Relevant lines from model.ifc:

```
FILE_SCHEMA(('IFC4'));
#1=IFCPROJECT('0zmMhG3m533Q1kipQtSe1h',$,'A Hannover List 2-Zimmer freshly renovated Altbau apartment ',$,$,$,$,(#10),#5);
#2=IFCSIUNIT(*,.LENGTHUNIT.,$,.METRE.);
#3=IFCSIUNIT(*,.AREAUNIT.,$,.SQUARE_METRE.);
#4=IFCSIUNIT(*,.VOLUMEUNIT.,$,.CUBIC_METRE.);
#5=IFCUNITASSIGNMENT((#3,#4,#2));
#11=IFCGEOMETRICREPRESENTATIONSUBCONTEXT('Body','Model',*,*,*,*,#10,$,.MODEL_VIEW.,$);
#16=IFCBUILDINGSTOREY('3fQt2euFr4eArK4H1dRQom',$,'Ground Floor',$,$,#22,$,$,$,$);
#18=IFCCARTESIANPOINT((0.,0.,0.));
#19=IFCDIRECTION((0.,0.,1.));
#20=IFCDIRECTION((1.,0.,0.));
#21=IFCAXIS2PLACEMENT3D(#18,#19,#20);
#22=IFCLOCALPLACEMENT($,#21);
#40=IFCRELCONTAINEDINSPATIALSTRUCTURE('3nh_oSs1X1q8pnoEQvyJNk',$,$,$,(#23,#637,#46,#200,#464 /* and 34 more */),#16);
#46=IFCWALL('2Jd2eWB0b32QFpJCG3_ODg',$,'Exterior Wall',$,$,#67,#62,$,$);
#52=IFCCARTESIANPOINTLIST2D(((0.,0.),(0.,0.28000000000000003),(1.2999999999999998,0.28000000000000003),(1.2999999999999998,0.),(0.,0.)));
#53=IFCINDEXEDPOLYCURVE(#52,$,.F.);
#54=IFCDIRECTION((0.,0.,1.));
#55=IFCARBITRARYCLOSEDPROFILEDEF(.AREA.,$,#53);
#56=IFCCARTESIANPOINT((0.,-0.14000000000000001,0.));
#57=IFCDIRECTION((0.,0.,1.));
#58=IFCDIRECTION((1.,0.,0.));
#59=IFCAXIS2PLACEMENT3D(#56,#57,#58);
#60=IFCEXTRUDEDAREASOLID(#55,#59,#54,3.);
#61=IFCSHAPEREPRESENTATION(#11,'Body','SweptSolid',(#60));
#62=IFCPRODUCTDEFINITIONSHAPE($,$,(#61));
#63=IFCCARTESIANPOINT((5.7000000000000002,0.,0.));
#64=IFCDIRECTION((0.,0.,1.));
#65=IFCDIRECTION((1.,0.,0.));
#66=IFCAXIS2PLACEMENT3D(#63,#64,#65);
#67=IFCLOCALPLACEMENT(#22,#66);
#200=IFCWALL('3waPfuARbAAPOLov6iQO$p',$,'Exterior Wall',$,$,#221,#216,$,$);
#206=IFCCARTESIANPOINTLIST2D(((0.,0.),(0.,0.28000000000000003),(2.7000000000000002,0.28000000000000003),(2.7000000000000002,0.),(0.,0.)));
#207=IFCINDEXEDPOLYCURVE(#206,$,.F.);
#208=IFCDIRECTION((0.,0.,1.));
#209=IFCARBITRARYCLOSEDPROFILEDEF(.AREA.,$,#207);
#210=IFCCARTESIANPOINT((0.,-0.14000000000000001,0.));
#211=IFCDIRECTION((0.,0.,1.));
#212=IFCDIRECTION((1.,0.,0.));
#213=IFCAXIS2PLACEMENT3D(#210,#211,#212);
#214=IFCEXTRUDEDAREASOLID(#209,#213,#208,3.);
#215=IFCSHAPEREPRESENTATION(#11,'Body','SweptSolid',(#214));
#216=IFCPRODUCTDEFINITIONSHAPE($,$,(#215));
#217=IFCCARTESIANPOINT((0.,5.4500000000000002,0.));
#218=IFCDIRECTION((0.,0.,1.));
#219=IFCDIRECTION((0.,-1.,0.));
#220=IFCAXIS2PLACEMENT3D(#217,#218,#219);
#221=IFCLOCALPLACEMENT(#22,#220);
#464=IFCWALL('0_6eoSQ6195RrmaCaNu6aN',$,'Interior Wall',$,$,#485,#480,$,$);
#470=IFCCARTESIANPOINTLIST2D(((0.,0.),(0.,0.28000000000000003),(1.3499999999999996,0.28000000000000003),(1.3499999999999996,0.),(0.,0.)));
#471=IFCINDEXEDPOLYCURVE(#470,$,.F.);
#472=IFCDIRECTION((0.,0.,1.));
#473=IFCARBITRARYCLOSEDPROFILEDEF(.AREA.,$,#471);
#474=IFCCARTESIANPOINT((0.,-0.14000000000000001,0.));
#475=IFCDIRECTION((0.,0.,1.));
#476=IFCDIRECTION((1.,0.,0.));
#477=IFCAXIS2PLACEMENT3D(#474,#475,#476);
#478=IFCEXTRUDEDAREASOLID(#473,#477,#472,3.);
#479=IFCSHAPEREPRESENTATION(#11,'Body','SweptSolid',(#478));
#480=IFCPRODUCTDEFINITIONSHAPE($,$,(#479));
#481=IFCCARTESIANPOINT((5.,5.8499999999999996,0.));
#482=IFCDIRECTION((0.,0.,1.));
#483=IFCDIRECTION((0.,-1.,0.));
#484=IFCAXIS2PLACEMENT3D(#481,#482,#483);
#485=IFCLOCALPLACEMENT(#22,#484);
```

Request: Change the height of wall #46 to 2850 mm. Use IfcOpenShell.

```python
import ifcopenshell
import ifcopenshell.geom
import ifcopenshell.util.representation
import ifcopenshell.util.shape

model = ifcopenshell.open("model.ifc")
settings = ifcopenshell.geom.settings()


def volume(element):
    """Net volume in cubic metres, openings subtracted."""
    shape = ifcopenshell.geom.create_shape(settings, element)
    return ifcopenshell.util.shape.get_volume(shape.geometry)


wall = model.by_id(46)
before = volume(wall)

body = ifcopenshell.util.representation.get_representation(wall, "Model", "Body")
solid = body.Items[0]
old_height = solid.Depth
solid.Depth = 2.85
after = volume(wall)

print(f"height {old_height:g} -> {solid.Depth:g}, volume {before:.3f} -> {after:.3f} m3")

model.write("model_v2.ifc")
```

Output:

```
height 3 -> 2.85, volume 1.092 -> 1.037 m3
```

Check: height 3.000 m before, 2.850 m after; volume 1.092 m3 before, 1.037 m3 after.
